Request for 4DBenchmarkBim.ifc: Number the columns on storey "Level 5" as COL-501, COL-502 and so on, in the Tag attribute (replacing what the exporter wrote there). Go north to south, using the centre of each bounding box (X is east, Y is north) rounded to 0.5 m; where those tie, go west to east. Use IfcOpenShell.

First a look at what the model holds.

```python
import ifcopenshell
import ifcopenshell.util.element
import ifcopenshell.util.placement

model = ifcopenshell.open("4DBenchmarkBim.ifc")
print(model.schema)
storey = next(s for s in model.by_type("IfcBuildingStorey") if s.Name == "Level 5")
columns = [e for e in ifcopenshell.util.element.get_decomposition(storey) if e.is_a("IfcColumn")]
for e in sorted(columns, key=lambda e: e.id()):
    origin = ifcopenshell.util.placement.get_local_placement(e.ObjectPlacement)[:3, 3]
    print(e.id(), e.Tag, e.Name, origin.round(2) + 0.0, sep=" | ")
```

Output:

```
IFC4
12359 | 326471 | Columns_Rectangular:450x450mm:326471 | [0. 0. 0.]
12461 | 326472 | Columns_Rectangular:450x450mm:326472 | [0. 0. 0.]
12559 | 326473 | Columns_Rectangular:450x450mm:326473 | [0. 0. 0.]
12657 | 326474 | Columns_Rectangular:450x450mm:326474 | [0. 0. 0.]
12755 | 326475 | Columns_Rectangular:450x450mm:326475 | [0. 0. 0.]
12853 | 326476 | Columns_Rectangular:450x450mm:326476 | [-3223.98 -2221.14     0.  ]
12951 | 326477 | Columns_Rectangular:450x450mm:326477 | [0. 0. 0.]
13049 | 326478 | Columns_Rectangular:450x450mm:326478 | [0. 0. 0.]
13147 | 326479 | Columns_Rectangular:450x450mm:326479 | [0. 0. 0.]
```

```python
import ifcopenshell
import ifcopenshell.geom
import ifcopenshell.util.element
import ifcopenshell.util.shape

model = ifcopenshell.open("4DBenchmarkBim.ifc")
settings = ifcopenshell.geom.settings()
settings.set("use-world-coords", True)


def centre(element):
    shape = ifcopenshell.geom.create_shape(settings, element)
    return ifcopenshell.util.shape.get_bbox_centroid(shape.geometry)


storey = next(s for s in model.by_type("IfcBuildingStorey") if s.Name == "Level 5")
columns = [e for e in ifcopenshell.util.element.get_decomposition(storey) if e.is_a("IfcColumn")]

# Insertion points can sit at a corner or the storey origin, so sort by the geometry (in metres).
centres = {e: centre(e) for e in columns}
columns.sort(key=lambda e: (-round(centres[e][1] / 0.5), centres[e][0]))

for i, e in enumerate(columns, start=1):
    number = f"COL-5{i:02d}"
    e.Tag = number
    print(e.id(), number)

model.write("4DBenchmarkBim_rev.ifc")
```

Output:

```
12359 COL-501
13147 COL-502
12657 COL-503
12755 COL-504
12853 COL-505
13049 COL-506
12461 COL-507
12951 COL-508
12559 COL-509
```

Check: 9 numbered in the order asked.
